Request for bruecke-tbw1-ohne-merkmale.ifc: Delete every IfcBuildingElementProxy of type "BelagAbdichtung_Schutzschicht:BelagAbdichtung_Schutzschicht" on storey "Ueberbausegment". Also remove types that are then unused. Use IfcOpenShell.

First a look at what the model holds.

```python
import ifcopenshell
import ifcopenshell.util.element

model = ifcopenshell.open("bruecke-tbw1-ohne-merkmale.ifc")
print(model.schema)
storey = next(s for s in model.by_type("IfcBuildingStorey") if s.Name == "Ueberbausegment")
proxies = [e for e in ifcopenshell.util.element.get_decomposition(storey) if e.is_a("IfcBuildingElementProxy")]
seen = {}
for e in proxies:
    element_type = ifcopenshell.util.element.get_type(e)
    name = element_type.Name if element_type not in (None, e) else None
    seen[name] = seen.get(name, 0) + 1
for name, count in sorted(seen.items(), key=str):
    print(count, "x", name)
```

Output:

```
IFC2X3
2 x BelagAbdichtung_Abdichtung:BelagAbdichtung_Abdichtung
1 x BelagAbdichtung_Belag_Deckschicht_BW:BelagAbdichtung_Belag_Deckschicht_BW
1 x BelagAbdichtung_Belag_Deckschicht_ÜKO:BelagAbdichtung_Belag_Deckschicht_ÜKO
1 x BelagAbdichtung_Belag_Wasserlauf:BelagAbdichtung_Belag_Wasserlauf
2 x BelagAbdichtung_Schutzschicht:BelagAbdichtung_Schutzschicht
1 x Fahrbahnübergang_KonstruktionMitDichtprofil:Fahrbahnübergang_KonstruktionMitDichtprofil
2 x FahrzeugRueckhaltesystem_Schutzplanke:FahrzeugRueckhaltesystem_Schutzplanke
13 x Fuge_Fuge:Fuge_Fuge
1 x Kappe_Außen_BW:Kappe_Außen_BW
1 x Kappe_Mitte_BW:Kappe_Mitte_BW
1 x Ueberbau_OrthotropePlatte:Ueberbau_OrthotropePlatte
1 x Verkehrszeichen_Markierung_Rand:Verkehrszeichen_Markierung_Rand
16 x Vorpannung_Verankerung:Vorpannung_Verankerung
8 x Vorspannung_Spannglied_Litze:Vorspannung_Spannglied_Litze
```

```python
import ifcopenshell
import ifcopenshell.api.root
import ifcopenshell.util.element

model = ifcopenshell.open("bruecke-tbw1-ohne-merkmale.ifc")

storey = next(s for s in model.by_type("IfcBuildingStorey") if s.Name == "Ueberbausegment")
proxies = [e for e in ifcopenshell.util.element.get_decomposition(storey) if e.is_a("IfcBuildingElementProxy")]
targets = [e for e in proxies if (t := ifcopenshell.util.element.get_type(e)) not in (None, e) and t.Name == "BelagAbdichtung_Schutzschicht:BelagAbdichtung_Schutzschicht"]
types = {ifcopenshell.util.element.get_type(e) for e in targets} - {None, *targets}

for e in targets:
    ifcopenshell.api.root.remove_product(model, product=e)
print(len(targets), "removed")

unused = [t for t in types if not ifcopenshell.util.element.get_types(t)]
for t in unused:
    ifcopenshell.api.root.remove_product(model, product=t)
print(len(unused), "unused types removed")

model.write("bruecke-tbw1-ohne-merkmale_updated.ifc")
```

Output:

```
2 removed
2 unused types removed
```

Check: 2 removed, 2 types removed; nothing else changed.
